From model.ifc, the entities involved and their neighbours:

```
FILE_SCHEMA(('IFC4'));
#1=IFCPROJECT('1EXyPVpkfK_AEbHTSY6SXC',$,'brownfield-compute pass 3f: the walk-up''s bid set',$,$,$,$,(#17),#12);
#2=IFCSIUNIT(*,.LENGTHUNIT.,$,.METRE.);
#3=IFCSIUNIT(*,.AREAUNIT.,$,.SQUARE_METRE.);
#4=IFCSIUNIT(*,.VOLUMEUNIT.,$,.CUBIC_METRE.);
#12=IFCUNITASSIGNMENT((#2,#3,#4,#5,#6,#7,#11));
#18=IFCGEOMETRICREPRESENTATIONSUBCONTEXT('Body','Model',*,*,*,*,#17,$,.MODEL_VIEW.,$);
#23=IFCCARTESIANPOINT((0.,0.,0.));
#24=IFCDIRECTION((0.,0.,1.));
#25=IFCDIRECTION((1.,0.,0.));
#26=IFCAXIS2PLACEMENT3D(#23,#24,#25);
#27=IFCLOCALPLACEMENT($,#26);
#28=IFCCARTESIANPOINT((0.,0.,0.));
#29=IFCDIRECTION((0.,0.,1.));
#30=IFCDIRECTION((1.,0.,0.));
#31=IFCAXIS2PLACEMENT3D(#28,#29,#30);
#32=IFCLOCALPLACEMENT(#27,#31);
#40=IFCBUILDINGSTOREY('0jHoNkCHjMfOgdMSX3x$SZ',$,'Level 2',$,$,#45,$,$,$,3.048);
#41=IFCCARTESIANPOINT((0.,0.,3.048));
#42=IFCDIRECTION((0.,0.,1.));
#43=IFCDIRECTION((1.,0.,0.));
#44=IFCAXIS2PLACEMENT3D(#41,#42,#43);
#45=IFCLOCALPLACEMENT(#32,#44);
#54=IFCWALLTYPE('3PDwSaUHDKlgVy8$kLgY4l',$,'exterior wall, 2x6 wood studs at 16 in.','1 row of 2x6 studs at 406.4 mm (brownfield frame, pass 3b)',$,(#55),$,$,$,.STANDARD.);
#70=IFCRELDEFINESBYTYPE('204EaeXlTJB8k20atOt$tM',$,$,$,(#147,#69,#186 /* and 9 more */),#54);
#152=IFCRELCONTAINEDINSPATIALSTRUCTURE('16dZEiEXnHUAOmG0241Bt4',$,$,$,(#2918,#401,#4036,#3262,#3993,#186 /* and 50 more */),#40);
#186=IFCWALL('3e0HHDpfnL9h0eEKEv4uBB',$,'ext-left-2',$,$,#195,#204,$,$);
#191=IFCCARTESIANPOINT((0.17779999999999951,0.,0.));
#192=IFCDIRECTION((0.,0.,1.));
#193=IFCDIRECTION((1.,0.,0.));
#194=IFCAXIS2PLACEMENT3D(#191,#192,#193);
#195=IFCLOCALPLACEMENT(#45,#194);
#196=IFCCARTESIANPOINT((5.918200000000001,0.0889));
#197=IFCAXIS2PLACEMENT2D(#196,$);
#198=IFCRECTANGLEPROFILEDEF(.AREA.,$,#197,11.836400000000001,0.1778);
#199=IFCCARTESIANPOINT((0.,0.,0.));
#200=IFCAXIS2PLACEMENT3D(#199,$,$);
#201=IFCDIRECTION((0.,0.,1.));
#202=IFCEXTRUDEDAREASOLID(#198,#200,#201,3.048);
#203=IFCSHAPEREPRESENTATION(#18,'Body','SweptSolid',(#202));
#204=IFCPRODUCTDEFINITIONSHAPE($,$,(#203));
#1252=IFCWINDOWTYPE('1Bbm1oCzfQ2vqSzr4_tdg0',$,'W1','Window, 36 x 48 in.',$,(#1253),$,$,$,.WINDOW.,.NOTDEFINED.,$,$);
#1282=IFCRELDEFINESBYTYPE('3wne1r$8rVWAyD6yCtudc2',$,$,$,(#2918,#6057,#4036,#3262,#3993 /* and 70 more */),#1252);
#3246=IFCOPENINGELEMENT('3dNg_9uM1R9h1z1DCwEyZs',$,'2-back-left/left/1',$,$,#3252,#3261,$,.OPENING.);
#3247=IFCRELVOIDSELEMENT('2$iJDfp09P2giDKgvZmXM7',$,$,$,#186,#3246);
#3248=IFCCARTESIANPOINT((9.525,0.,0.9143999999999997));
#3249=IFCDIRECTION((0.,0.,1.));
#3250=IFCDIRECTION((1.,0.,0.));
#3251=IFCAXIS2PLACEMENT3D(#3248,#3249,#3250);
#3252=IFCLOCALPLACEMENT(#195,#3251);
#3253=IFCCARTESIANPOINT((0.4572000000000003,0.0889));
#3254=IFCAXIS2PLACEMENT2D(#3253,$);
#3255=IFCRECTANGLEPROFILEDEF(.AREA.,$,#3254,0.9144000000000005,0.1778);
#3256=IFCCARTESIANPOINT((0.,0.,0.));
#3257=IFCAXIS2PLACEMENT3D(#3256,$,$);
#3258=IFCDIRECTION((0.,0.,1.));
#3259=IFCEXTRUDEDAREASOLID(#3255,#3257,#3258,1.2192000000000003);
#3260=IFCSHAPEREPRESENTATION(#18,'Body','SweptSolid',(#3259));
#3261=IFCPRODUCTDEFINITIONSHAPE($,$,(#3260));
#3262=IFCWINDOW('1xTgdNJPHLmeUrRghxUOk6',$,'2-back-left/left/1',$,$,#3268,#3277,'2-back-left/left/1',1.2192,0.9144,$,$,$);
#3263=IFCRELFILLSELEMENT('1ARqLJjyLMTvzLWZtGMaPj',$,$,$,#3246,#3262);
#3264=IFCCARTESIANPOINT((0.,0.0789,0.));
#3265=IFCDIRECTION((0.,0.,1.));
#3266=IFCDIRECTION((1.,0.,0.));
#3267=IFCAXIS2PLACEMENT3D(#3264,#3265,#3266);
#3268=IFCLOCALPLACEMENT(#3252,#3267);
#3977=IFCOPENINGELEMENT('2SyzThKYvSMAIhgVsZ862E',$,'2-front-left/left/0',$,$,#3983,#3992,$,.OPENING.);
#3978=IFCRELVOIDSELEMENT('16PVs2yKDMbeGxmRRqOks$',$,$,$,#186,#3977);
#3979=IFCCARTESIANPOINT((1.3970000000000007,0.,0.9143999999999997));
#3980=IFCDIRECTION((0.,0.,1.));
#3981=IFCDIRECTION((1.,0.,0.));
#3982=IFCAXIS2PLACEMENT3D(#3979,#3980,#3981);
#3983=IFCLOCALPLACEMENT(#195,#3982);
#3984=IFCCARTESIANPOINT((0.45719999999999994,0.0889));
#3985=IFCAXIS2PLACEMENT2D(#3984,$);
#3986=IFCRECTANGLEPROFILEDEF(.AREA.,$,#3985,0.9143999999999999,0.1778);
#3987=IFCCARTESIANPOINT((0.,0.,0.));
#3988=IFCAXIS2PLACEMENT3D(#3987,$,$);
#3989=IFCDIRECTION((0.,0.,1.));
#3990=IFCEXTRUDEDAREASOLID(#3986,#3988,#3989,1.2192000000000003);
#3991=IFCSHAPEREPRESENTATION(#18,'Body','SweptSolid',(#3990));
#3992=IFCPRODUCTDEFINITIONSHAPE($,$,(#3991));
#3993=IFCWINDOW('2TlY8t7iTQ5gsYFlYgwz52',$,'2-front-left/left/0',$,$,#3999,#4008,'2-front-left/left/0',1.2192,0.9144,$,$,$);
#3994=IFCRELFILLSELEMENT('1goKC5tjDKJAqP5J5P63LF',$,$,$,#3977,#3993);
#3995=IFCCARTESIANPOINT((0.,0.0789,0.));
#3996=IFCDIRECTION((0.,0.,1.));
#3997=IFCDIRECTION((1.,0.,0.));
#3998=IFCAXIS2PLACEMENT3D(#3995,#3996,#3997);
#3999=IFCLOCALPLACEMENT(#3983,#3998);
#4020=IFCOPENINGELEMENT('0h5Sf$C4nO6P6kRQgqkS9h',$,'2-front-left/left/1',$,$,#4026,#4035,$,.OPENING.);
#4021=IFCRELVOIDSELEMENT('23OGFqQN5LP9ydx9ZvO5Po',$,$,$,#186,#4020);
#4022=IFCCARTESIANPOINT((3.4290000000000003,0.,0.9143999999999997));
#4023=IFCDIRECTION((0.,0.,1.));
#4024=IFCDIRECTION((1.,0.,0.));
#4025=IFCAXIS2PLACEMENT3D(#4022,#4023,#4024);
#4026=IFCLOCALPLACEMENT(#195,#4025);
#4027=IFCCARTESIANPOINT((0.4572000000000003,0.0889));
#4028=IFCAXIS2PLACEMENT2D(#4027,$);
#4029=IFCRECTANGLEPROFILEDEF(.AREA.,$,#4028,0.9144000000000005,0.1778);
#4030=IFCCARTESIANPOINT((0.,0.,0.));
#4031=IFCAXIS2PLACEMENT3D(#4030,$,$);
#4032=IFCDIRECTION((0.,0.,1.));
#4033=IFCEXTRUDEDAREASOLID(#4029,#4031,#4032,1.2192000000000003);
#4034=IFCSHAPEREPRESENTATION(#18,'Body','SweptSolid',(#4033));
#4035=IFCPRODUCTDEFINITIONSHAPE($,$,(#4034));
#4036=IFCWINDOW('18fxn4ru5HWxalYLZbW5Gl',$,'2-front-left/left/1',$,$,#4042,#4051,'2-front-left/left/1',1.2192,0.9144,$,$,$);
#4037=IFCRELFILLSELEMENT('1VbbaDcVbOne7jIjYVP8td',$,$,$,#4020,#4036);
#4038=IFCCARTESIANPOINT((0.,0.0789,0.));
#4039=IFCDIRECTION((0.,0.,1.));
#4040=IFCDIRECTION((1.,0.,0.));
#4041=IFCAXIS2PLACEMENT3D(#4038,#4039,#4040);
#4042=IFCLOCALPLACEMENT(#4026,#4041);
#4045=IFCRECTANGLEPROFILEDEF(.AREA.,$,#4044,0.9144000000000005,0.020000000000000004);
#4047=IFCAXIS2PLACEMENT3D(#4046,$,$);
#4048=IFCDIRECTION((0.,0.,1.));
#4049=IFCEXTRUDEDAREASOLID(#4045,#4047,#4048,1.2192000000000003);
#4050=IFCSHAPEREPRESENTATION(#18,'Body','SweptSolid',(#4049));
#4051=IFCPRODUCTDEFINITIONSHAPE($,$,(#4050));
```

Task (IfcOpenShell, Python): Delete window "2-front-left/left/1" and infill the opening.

```python
import ifcopenshell
import ifcopenshell.api.feature
import ifcopenshell.api.root
import ifcopenshell.geom
import ifcopenshell.util.shape

model = ifcopenshell.open("model.ifc")
settings = ifcopenshell.geom.settings()


def volume(element):
    """Net volume in cubic metres, openings subtracted."""
    shape = ifcopenshell.geom.create_shape(settings, element)
    return ifcopenshell.util.shape.get_volume(shape.geometry)


window = model.by_guid("18fxn4ru5HWxalYLZbW5Gl")
opening = window.FillsVoids[0].RelatingOpeningElement
wall = opening.VoidsElements[0].RelatingBuildingElement
before = volume(wall)

ifcopenshell.api.root.remove_product(model, product=window)
ifcopenshell.api.feature.remove_feature(model, feature=opening)

after = volume(wall)

print(f"wall volume {before:.3f} -> {after:.3f} m3")

model.write("model_v2.ifc")
```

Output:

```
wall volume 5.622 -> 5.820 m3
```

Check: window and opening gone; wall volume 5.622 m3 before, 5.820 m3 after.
